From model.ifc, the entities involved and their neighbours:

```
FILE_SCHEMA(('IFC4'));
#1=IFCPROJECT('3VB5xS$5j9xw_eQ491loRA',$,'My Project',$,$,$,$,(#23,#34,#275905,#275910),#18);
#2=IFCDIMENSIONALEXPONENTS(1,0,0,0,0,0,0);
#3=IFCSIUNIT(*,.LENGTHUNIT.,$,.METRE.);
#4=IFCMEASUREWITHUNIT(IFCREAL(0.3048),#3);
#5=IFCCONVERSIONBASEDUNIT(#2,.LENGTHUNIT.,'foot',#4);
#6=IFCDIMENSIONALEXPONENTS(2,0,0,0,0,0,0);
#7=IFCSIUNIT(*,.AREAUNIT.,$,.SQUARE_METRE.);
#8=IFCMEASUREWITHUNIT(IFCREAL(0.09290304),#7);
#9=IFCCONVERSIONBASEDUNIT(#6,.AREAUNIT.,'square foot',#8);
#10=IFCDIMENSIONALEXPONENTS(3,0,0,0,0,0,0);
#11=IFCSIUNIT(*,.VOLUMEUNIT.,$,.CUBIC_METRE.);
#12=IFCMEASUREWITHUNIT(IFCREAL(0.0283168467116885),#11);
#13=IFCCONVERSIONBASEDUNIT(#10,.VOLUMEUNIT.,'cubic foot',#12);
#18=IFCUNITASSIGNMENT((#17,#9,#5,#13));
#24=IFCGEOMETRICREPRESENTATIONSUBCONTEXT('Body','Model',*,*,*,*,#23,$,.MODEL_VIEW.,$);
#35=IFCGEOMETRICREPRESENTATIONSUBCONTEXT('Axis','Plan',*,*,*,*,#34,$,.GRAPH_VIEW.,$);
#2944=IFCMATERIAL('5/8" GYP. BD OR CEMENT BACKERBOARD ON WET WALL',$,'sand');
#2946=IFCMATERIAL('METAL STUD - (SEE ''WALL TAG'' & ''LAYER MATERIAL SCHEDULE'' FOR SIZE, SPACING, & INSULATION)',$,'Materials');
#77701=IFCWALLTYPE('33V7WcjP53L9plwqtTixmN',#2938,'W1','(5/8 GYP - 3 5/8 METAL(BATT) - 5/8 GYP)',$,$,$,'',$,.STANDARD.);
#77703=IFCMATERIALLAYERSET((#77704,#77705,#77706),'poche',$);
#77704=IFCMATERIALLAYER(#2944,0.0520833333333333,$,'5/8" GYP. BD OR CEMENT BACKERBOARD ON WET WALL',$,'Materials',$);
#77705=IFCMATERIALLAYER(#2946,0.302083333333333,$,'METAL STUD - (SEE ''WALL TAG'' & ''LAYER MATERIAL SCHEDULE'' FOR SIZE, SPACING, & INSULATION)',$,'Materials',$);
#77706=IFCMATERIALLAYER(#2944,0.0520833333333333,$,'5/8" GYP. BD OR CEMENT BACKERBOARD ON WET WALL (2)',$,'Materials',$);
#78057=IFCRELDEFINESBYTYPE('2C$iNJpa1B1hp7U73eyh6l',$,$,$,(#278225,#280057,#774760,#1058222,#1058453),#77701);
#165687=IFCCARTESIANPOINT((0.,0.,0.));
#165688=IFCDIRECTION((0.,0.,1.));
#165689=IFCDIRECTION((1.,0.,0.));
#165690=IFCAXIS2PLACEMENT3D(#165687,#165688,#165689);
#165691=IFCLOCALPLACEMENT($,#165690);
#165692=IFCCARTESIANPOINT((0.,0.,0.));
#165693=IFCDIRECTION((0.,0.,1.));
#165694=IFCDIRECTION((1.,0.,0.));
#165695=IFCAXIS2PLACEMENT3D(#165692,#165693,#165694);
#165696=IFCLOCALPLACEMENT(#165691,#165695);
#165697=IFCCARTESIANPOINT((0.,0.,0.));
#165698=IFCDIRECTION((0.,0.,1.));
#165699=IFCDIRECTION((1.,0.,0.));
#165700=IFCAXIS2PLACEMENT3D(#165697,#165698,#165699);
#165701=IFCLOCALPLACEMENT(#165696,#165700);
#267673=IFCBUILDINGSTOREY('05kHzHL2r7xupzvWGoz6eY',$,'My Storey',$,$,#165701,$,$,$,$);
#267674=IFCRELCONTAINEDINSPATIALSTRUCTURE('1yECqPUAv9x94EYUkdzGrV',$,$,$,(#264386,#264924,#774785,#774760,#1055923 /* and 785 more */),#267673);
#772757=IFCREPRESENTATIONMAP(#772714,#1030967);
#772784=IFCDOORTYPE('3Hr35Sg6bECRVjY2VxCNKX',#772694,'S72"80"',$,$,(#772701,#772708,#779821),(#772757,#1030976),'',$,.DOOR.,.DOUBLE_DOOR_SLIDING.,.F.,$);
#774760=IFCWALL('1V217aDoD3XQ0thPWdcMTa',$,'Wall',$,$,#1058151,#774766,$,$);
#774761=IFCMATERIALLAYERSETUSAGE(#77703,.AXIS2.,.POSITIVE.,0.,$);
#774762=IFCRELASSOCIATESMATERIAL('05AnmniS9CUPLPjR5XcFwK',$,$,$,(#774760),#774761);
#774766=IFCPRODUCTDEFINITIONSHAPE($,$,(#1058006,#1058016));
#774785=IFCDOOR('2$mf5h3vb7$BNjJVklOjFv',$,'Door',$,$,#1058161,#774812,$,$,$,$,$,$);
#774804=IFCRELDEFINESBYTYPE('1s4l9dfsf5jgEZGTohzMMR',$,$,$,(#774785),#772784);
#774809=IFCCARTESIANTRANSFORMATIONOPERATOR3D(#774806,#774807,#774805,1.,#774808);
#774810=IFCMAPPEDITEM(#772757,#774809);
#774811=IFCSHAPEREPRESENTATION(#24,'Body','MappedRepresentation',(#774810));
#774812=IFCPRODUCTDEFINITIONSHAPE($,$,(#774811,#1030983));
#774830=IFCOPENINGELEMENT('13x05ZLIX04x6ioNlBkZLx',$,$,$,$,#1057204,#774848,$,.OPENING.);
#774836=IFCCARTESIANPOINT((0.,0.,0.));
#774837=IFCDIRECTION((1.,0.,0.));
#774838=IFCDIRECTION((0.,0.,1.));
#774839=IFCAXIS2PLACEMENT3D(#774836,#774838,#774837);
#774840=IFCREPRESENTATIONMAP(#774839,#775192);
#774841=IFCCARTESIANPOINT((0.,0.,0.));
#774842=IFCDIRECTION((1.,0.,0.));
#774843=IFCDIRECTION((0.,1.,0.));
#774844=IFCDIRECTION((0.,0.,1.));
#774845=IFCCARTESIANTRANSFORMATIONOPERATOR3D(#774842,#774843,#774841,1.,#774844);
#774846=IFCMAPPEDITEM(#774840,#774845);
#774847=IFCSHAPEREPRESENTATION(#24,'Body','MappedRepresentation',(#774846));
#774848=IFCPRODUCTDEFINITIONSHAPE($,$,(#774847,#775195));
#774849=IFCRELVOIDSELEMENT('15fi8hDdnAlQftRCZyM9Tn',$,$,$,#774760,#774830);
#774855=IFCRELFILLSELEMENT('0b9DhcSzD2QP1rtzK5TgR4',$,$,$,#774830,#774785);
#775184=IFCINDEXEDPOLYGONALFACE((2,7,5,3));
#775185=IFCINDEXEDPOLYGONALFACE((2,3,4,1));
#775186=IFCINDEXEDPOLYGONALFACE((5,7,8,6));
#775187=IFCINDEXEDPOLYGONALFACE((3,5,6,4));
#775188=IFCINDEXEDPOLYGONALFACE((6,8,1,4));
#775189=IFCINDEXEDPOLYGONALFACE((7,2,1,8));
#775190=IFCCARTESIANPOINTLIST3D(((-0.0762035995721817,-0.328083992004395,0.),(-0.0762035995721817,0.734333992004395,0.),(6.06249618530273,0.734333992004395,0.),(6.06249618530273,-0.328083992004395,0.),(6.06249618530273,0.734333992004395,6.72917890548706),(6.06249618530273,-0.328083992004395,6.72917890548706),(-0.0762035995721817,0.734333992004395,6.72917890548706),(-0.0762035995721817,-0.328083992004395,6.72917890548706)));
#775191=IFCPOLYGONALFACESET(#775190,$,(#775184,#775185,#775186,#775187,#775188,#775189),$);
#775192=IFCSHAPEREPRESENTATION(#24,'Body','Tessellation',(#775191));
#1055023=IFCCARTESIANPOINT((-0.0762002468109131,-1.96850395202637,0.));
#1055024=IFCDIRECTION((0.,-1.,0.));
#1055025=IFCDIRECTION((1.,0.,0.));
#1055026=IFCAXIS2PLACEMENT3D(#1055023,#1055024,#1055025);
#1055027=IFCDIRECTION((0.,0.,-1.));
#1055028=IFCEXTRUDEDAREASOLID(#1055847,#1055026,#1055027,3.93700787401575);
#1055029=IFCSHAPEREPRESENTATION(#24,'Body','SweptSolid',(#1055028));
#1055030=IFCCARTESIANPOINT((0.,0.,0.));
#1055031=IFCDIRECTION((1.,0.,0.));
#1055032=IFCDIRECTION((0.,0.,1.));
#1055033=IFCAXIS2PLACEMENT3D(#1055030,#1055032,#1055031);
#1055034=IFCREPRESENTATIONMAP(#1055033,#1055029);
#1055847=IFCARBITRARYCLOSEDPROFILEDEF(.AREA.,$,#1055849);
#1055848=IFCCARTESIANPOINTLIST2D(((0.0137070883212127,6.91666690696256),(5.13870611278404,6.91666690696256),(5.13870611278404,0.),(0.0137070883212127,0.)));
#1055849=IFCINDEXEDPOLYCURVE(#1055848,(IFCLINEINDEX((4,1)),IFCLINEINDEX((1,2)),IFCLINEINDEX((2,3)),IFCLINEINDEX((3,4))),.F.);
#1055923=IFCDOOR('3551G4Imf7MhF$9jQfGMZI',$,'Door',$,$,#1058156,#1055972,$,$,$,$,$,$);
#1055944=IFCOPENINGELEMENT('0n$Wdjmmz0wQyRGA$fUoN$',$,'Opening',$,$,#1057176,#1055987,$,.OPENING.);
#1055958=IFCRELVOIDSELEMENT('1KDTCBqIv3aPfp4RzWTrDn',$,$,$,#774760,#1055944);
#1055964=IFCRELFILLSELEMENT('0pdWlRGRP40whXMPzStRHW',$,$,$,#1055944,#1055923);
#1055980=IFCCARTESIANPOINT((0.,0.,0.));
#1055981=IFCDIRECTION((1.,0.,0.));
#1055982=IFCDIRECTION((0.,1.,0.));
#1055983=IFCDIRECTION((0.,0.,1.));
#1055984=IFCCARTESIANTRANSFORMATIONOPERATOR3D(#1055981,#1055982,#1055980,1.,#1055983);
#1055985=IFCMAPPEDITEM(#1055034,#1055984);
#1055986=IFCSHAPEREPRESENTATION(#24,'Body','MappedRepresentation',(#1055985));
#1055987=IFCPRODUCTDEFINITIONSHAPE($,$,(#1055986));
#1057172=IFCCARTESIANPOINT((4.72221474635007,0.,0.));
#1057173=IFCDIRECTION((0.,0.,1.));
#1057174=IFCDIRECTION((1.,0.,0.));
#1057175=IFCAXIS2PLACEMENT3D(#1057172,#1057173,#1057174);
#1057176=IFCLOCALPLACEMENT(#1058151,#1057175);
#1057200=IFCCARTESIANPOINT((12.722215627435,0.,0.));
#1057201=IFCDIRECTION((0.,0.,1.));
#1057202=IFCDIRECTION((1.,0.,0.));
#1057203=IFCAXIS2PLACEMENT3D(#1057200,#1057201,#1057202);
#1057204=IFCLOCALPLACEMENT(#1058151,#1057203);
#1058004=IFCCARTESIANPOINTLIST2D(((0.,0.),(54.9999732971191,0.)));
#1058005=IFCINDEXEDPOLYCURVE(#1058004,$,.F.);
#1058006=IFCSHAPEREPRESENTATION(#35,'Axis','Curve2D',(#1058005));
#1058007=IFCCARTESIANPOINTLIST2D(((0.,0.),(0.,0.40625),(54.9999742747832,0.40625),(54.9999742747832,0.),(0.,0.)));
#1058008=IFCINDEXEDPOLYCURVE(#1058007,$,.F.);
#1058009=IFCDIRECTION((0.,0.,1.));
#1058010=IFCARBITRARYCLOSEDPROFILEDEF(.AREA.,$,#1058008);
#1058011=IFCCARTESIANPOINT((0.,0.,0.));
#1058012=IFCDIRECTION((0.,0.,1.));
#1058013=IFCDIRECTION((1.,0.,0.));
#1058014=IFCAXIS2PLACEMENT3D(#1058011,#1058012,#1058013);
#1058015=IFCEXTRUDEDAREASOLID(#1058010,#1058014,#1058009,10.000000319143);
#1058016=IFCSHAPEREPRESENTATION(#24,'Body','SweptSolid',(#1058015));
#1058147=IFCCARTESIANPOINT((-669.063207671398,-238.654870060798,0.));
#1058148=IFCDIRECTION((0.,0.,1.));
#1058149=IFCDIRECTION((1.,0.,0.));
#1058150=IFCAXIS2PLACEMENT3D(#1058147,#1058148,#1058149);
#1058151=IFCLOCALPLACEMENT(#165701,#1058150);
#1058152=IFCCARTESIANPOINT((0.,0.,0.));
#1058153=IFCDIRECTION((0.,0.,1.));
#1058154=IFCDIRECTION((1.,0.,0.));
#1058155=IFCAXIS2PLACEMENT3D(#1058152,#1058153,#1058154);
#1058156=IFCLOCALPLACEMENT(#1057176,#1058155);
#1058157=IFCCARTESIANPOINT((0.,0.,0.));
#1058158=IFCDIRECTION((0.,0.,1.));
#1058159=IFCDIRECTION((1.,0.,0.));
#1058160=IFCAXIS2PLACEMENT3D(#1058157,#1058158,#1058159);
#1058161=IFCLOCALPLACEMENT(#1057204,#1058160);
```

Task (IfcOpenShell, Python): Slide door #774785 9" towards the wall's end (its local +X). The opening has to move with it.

```python
import ifcopenshell
import ifcopenshell.api.geometry
import ifcopenshell.util.placement
import ifcopenshell.util.unit

model = ifcopenshell.open("model.ifc")
unit_scale = ifcopenshell.util.unit.calculate_unit_scale(model)

door = model.by_id(774785)
opening = door.FillsVoids[0].RelatingOpeningElement
wall = opening.VoidsElements[0].RelatingBuildingElement

wall_matrix = ifcopenshell.util.placement.get_local_placement(wall.ObjectPlacement)
shift = wall_matrix[:3, 0] * 9 * 0.0254 / unit_scale
before = ifcopenshell.util.placement.get_local_placement(door.ObjectPlacement)[:3, 3].copy()

# The door is placed relative to its opening, so it follows when the opening moves.
matrix = ifcopenshell.util.placement.get_local_placement(opening.ObjectPlacement)
matrix[:3, 3] += shift
ifcopenshell.api.geometry.edit_object_placement(
    model, product=opening, matrix=matrix, is_si=False, should_transform_children=True
)

after = ifcopenshell.util.placement.get_local_placement(door.ObjectPlacement)[:3, 3]
print("door moved by", (after - before).round(3) + 0.0)

model.write("model_v2.ifc")
```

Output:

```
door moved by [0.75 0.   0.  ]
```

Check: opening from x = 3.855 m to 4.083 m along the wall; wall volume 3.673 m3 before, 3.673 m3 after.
